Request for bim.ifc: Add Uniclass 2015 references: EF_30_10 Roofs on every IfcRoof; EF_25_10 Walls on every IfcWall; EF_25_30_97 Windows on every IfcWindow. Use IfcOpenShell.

First a look at what the model holds.

```python
import ifcopenshell

model = ifcopenshell.open("bim.ifc")
print(model.schema)
print("classifications:", [c.Name for c in model.by_type("IfcClassification")])
for ifc_class in ("IfcDoor", "IfcRoof", "IfcStair", "IfcWall", "IfcWindow"):
    print(ifc_class, len(model.by_type(ifc_class)))
```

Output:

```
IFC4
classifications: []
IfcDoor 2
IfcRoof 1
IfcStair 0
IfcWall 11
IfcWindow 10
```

```python
import ifcopenshell
import ifcopenshell.api.classification

model = ifcopenshell.open("bim.ifc")

system = ifcopenshell.api.classification.add_classification(model, classification="Uniclass 2015")

codes = {
    "IfcRoof": ("EF_30_10", "Roofs"),
    "IfcWall": ("EF_25_10", "Walls"),
    "IfcWindow": ("EF_25_30_97", "Windows"),
}
for ifc_class, (code, name) in codes.items():
    products = model.by_type(ifc_class)
    ifcopenshell.api.classification.add_reference(
        model, products=products, classification=system, identification=code, name=name
    )
    print(code, len(products))

model.write("bim_rev.ifc")
```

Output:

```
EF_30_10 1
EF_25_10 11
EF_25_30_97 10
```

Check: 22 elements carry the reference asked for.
